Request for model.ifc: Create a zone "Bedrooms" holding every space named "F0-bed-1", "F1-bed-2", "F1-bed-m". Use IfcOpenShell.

First a look at what the model holds.

```python
import ifcopenshell

model = ifcopenshell.open("model.ifc")
print(model.schema)
seen = {}
for space in model.by_type("IfcSpace"):
    seen[space.LongName] = seen.get(space.LongName, 0) + 1
for name, count in sorted(seen.items(), key=str):
    print(count, "x", name)
print("zones:", [z.Name for z in model.by_type("IfcZone")][:20])
```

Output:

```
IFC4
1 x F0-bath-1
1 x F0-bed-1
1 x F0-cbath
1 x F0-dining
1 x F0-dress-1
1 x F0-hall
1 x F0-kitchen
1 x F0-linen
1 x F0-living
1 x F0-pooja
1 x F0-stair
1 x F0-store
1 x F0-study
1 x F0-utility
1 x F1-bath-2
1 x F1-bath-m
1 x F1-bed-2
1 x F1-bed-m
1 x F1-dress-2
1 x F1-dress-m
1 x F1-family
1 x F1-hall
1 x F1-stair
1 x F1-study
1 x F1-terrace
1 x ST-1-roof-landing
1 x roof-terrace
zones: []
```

```python
import ifcopenshell
import ifcopenshell.api.group
import ifcopenshell.api.root

model = ifcopenshell.open("model.ifc")

names = {"F0-bed-1", "F1-bed-2", "F1-bed-m"}
spaces = [s for s in model.by_type("IfcSpace") if s.LongName in names]

zone = ifcopenshell.api.root.create_entity(model, ifc_class="IfcZone", name="Bedrooms")
ifcopenshell.api.group.assign_group(model, products=spaces, group=zone)
print(len(spaces), "spaces in", zone.Name)

model.write("model_edited.ifc")
```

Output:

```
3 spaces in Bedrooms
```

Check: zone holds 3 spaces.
